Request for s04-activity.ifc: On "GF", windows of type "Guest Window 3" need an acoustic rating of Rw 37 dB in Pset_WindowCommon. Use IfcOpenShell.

First a look at what the model holds.

```python
import ifcopenshell
import ifcopenshell.util.element

model = ifcopenshell.open("s04-activity.ifc")
print(model.schema)
storey = next(s for s in model.by_type("IfcBuildingStorey") if s.Name == "GF")
windows = [e for e in ifcopenshell.util.element.get_decomposition(storey) if e.is_a("IfcWindow")]
seen = {}
for e in windows:
    element_type = ifcopenshell.util.element.get_type(e)
    key = (element_type.Name if element_type != e and element_type else None, ifcopenshell.util.element.get_pset(e, "Pset_WindowCommon", "AcousticRating"))
    seen[key] = seen.get(key, 0) + 1
for (name, value), count in sorted(seen.items(), key=str):
    print(count, "x", name, "|", value)
```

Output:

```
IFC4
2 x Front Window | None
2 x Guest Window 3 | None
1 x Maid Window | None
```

```python
import ifcopenshell
import ifcopenshell.api.pset
import ifcopenshell.util.element

model = ifcopenshell.open("s04-activity.ifc")

storey = next(s for s in model.by_type("IfcBuildingStorey") if s.Name == "GF")
windows = [e for e in ifcopenshell.util.element.get_decomposition(storey) if e.is_a("IfcWindow")]

count = 0
for e in windows:
    element_type = ifcopenshell.util.element.get_type(e)
    if element_type in (None, e) or element_type.Name != "Guest Window 3":
        continue
    # add_pset returns the element's existing set when there is one.
    pset = ifcopenshell.api.pset.add_pset(model, product=e, name="Pset_WindowCommon")
    ifcopenshell.api.pset.edit_pset(model, pset=pset, properties={"AcousticRating": "Rw 37 dB"})
    count += 1

print(count, "windows updated")

model.write("s04-activity_edited.ifc")
```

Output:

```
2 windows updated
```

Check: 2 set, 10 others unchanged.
